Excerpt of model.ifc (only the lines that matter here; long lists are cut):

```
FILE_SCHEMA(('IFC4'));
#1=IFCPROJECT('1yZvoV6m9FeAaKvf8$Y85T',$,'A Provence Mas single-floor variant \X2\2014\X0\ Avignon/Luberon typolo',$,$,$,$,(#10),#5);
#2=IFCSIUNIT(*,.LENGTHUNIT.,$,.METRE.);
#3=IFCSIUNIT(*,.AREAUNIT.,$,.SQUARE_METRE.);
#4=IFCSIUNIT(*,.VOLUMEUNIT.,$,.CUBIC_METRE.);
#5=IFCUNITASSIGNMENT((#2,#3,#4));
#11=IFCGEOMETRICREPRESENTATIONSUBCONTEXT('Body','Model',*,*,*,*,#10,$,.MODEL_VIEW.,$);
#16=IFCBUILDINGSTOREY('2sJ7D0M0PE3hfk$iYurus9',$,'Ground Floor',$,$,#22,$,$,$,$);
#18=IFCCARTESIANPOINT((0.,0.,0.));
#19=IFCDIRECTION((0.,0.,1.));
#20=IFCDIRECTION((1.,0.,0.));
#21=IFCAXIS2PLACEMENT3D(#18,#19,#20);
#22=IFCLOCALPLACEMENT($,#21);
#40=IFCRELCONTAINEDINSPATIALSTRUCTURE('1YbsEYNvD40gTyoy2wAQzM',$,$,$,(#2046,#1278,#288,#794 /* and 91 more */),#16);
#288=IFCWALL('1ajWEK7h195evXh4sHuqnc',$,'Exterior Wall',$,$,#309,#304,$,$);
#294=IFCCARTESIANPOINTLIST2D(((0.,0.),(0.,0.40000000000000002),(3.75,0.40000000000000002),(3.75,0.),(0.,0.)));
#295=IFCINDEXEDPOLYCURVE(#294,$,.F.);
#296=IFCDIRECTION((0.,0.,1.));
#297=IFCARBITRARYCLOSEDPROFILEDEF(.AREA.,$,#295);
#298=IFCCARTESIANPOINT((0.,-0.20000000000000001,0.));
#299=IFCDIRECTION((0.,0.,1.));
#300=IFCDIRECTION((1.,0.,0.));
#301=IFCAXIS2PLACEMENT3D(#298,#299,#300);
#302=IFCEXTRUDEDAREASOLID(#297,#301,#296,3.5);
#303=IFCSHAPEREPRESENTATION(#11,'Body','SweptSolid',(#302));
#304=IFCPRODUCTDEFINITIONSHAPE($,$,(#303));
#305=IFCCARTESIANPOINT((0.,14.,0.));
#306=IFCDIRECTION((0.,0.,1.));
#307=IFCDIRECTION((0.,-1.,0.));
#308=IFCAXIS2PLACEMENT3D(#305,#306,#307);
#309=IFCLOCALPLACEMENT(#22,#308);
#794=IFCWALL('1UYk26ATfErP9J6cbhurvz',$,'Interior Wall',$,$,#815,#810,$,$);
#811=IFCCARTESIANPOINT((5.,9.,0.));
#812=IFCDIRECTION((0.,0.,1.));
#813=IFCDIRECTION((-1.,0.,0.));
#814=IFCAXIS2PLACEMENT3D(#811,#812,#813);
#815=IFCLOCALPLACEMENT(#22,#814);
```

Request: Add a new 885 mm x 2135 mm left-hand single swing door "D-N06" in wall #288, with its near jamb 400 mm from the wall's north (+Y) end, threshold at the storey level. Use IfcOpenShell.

```python
import numpy as np
import ifcopenshell
import ifcopenshell.api.feature
import ifcopenshell.api.geometry
import ifcopenshell.api.root
import ifcopenshell.api.spatial
import ifcopenshell.geom
import ifcopenshell.util.element
import ifcopenshell.util.placement
import ifcopenshell.util.representation
import ifcopenshell.util.shape
import ifcopenshell.util.unit

model = ifcopenshell.open("model.ifc")
unit_scale = ifcopenshell.util.unit.calculate_unit_scale(model)
settings = ifcopenshell.geom.settings()


def volume(element):
    """Net volume in cubic metres, openings subtracted."""
    shape = ifcopenshell.geom.create_shape(settings, element)
    return ifcopenshell.util.shape.get_volume(shape.geometry)


wall = model.by_guid("1ajWEK7h195evXh4sHuqnc")
storey = ifcopenshell.util.element.get_container(wall, ifc_class="IfcBuildingStorey")
context = ifcopenshell.util.representation.get_context(model, "Model", "Body", "MODEL_VIEW")
before = volume(wall)

width, height, from_end, sill = 0.885, 2.135, 0.4, 0.0  # metres

# The wall runs along its own X axis, and the end named is its -X end.
wall_shape = ifcopenshell.geom.create_shape(settings, wall)
x, y, z = ifcopenshell.util.shape.get_vertices(wall_shape.geometry).T
start = x.min() + from_end
face, thickness = float(y.min()), float(y.max() - y.min())
wall_matrix = ifcopenshell.util.placement.get_local_placement(wall.ObjectPlacement)
level = ifcopenshell.util.placement.get_local_placement(storey.ObjectPlacement)[2, 3]


def in_wall(x, y):
    """Placement at x, y metres in the wall's axes, at sill height."""
    matrix = wall_matrix.copy()
    matrix[:, 3] = wall_matrix @ np.array([x / unit_scale, y / unit_scale, 0.0, 1.0])
    matrix[2, 3] = level + sill / unit_scale
    return matrix


# Opening: a box that overshoots both wall faces by 50 mm.
opening = ifcopenshell.api.root.create_entity(model, ifc_class="IfcOpeningElement", predefined_type="OPENING")
box = ifcopenshell.api.geometry.add_wall_representation(
    model, context=context, length=width, height=height, thickness=thickness + 0.1
)
ifcopenshell.api.geometry.assign_representation(model, product=opening, representation=box)
ifcopenshell.api.geometry.edit_object_placement(model, product=opening, matrix=in_wall(start, face - 0.05), is_si=False)
ifcopenshell.api.feature.add_feature(model, feature=opening, element=wall)

door = ifcopenshell.api.root.create_entity(model, ifc_class="IfcDoor", name="D-N06", predefined_type="DOOR")
door.OverallWidth, door.OverallHeight = width / unit_scale, height / unit_scale
door.OperationType = "SINGLE_SWING_LEFT"
body = ifcopenshell.api.geometry.add_door_representation(
    model,
    context=context,
    overall_width=door.OverallWidth,
    overall_height=door.OverallHeight,
    operation_type="SINGLE_SWING_LEFT",
    lining_properties={"LiningDepth": thickness / unit_scale, "ThresholdDepth": thickness / unit_scale},
)
ifcopenshell.api.geometry.assign_representation(model, product=door, representation=body)
ifcopenshell.api.spatial.assign_container(model, products=[door], relating_structure=storey)
ifcopenshell.api.feature.add_filling(model, opening=opening, element=door)

# The lining spans the wall, so the door starts at the wall face.
ifcopenshell.api.geometry.edit_object_placement(model, product=door, matrix=in_wall(start, face), is_si=False)

after = volume(wall)

print(f"wall volume {before:.3f} -> {after:.3f} m3")

model.write("model_v2.ifc")
```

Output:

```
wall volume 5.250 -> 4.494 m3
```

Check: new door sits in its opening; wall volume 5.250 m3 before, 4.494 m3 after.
